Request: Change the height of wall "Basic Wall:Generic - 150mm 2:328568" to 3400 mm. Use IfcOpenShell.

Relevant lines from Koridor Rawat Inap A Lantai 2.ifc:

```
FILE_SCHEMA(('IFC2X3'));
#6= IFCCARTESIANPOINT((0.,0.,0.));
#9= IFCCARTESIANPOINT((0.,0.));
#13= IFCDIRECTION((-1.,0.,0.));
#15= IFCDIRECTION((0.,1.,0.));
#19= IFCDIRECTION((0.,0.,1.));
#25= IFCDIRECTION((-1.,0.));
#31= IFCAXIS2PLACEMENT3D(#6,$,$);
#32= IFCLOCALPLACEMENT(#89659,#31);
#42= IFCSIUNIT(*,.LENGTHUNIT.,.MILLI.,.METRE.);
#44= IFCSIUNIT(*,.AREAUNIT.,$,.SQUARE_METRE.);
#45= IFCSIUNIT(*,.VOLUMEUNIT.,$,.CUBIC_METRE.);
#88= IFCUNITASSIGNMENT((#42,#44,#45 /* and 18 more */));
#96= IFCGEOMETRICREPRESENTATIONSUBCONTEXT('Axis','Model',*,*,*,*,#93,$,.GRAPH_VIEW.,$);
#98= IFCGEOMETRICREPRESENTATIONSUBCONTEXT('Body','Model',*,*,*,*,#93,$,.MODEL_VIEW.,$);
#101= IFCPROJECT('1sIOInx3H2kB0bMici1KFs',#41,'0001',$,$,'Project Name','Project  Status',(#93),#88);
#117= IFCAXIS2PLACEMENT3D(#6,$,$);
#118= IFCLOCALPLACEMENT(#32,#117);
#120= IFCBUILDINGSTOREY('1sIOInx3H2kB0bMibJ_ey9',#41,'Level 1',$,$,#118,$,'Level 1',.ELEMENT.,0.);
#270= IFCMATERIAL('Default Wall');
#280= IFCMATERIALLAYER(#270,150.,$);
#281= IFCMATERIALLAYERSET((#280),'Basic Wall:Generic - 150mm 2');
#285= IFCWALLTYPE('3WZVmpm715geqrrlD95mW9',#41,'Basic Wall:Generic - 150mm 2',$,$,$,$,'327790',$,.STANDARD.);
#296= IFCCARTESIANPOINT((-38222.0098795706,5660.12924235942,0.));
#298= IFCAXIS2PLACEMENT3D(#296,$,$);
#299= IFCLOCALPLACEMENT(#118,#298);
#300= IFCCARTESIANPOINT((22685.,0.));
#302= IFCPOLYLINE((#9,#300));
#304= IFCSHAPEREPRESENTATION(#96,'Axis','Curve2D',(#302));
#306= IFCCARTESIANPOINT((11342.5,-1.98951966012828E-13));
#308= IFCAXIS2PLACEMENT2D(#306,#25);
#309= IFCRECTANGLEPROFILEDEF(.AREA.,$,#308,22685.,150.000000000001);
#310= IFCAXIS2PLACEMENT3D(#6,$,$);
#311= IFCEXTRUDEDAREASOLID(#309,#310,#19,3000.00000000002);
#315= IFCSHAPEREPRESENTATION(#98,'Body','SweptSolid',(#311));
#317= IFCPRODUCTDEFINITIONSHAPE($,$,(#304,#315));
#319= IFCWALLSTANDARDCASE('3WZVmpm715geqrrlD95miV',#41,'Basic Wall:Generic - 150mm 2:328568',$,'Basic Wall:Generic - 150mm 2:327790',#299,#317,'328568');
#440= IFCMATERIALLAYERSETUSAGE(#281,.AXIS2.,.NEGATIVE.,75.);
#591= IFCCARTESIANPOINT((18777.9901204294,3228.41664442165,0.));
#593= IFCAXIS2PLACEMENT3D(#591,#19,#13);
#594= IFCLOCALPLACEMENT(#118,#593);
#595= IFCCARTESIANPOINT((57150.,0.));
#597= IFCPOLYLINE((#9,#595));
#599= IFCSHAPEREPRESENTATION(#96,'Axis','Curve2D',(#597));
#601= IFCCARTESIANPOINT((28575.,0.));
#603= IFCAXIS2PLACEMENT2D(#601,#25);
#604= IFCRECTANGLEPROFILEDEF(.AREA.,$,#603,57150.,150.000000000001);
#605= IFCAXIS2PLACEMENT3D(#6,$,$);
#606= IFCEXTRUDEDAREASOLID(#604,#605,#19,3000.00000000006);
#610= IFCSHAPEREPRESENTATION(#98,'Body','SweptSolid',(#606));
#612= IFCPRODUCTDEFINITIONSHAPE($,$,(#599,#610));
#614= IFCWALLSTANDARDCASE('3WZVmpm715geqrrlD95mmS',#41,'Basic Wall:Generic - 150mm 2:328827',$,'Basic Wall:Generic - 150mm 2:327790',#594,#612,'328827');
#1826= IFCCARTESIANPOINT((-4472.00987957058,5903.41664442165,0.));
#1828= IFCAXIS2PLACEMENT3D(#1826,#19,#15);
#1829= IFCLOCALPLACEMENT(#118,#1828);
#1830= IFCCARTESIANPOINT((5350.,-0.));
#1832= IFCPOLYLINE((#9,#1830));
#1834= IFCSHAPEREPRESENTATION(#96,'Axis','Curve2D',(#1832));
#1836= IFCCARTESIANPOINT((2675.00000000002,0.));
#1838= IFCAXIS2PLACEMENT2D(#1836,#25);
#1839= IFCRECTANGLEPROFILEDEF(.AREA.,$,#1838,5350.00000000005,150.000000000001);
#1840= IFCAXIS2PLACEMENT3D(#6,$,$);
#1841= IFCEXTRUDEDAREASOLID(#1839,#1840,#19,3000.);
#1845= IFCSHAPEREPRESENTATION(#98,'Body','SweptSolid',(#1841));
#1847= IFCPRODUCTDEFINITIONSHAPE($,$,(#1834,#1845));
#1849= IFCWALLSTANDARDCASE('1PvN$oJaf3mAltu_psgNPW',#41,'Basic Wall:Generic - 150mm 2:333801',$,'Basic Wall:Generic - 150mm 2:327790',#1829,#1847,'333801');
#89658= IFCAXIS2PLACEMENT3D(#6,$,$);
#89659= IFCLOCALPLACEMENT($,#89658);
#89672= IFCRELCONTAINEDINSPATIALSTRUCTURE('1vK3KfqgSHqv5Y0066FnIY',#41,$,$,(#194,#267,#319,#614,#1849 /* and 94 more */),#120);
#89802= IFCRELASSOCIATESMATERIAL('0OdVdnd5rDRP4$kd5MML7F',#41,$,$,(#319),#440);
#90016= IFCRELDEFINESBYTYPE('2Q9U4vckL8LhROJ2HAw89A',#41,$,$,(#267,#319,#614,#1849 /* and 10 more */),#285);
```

```python
import ifcopenshell
import ifcopenshell.geom
import ifcopenshell.util.representation
import ifcopenshell.util.shape
import ifcopenshell.util.unit

model = ifcopenshell.open("Koridor Rawat Inap A Lantai 2.ifc")
unit_scale = ifcopenshell.util.unit.calculate_unit_scale(model)
settings = ifcopenshell.geom.settings()


def volume(element):
    """Net volume in cubic metres, openings subtracted."""
    shape = ifcopenshell.geom.create_shape(settings, element)
    return ifcopenshell.util.shape.get_volume(shape.geometry)


wall = model.by_guid("3WZVmpm715geqrrlD95miV")
before = volume(wall)

body = ifcopenshell.util.representation.get_representation(wall, "Model", "Body")
solid = body.Items[0]
old_height = solid.Depth
solid.Depth = 3.4 / unit_scale
after = volume(wall)

print(f"height {old_height:g} -> {solid.Depth:g}, volume {before:.3f} -> {after:.3f} m3")

model.write("Koridor Rawat Inap A Lantai 2_updated.ifc")
```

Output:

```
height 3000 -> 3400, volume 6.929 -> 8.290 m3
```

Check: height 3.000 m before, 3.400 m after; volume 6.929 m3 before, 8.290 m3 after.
